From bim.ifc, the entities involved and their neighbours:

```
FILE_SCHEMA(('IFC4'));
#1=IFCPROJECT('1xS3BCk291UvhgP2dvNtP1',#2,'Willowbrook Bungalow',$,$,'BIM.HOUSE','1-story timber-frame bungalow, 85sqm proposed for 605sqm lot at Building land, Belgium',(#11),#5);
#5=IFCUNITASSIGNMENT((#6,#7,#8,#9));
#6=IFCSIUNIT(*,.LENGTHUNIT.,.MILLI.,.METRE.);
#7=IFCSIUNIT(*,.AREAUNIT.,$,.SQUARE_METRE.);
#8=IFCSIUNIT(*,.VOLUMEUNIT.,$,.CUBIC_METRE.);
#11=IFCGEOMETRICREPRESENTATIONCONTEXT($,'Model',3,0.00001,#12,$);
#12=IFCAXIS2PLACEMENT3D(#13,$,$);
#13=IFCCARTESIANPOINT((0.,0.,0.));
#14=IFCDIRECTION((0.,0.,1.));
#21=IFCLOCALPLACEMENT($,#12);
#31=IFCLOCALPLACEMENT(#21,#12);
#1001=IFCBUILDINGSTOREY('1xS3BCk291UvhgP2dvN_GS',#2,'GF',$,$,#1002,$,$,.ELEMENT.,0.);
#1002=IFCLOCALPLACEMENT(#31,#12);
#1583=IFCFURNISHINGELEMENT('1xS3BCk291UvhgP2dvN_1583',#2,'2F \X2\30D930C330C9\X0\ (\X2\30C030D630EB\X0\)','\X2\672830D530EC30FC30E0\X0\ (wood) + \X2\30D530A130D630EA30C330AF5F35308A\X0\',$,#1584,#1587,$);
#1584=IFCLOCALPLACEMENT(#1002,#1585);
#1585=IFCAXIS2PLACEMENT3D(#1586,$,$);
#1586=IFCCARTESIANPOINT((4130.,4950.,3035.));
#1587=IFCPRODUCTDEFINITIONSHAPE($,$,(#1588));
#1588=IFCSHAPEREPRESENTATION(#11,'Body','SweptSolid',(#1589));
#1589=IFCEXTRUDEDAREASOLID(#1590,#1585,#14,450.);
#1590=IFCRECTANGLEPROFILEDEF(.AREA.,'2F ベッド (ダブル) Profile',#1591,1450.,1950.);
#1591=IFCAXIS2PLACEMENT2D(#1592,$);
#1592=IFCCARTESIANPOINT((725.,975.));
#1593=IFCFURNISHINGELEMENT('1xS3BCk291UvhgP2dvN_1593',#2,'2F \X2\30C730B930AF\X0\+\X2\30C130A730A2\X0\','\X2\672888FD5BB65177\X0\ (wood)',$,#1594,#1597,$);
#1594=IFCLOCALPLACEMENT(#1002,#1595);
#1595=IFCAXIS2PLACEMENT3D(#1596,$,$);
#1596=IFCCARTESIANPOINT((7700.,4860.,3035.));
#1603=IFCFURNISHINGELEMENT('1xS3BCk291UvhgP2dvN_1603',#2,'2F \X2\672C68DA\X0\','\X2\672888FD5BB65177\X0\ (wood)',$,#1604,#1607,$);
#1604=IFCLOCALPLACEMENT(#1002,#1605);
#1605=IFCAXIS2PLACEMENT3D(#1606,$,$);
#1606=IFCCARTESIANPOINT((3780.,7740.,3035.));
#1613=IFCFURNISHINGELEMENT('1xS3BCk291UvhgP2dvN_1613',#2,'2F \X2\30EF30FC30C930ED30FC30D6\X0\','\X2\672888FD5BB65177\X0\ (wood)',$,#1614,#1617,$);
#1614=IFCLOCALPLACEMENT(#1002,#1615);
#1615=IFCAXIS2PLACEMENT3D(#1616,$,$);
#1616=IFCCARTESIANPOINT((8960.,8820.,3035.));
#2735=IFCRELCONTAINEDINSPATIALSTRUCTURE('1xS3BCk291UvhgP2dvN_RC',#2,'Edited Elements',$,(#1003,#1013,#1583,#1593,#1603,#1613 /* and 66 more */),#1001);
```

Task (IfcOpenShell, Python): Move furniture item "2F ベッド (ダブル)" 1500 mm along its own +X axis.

```python
import ifcopenshell
import ifcopenshell.api.geometry
import ifcopenshell.util.placement

model = ifcopenshell.open("bim.ifc")

item = model.by_guid("1xS3BCk291UvhgP2dvN_1583")
matrix = ifcopenshell.util.placement.get_local_placement(item.ObjectPlacement)
matrix[:3, 3] += matrix[:3, 0] * 1500.0
ifcopenshell.api.geometry.edit_object_placement(model, product=item, matrix=matrix, is_si=False)

print(ifcopenshell.util.placement.get_local_placement(item.ObjectPlacement).round(3) + 0.0)

model.write("bim_edited.ifc")
```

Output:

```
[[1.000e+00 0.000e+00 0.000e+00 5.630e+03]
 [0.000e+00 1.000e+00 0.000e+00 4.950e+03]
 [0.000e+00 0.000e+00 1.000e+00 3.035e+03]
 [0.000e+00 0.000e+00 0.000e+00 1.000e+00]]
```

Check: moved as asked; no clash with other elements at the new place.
